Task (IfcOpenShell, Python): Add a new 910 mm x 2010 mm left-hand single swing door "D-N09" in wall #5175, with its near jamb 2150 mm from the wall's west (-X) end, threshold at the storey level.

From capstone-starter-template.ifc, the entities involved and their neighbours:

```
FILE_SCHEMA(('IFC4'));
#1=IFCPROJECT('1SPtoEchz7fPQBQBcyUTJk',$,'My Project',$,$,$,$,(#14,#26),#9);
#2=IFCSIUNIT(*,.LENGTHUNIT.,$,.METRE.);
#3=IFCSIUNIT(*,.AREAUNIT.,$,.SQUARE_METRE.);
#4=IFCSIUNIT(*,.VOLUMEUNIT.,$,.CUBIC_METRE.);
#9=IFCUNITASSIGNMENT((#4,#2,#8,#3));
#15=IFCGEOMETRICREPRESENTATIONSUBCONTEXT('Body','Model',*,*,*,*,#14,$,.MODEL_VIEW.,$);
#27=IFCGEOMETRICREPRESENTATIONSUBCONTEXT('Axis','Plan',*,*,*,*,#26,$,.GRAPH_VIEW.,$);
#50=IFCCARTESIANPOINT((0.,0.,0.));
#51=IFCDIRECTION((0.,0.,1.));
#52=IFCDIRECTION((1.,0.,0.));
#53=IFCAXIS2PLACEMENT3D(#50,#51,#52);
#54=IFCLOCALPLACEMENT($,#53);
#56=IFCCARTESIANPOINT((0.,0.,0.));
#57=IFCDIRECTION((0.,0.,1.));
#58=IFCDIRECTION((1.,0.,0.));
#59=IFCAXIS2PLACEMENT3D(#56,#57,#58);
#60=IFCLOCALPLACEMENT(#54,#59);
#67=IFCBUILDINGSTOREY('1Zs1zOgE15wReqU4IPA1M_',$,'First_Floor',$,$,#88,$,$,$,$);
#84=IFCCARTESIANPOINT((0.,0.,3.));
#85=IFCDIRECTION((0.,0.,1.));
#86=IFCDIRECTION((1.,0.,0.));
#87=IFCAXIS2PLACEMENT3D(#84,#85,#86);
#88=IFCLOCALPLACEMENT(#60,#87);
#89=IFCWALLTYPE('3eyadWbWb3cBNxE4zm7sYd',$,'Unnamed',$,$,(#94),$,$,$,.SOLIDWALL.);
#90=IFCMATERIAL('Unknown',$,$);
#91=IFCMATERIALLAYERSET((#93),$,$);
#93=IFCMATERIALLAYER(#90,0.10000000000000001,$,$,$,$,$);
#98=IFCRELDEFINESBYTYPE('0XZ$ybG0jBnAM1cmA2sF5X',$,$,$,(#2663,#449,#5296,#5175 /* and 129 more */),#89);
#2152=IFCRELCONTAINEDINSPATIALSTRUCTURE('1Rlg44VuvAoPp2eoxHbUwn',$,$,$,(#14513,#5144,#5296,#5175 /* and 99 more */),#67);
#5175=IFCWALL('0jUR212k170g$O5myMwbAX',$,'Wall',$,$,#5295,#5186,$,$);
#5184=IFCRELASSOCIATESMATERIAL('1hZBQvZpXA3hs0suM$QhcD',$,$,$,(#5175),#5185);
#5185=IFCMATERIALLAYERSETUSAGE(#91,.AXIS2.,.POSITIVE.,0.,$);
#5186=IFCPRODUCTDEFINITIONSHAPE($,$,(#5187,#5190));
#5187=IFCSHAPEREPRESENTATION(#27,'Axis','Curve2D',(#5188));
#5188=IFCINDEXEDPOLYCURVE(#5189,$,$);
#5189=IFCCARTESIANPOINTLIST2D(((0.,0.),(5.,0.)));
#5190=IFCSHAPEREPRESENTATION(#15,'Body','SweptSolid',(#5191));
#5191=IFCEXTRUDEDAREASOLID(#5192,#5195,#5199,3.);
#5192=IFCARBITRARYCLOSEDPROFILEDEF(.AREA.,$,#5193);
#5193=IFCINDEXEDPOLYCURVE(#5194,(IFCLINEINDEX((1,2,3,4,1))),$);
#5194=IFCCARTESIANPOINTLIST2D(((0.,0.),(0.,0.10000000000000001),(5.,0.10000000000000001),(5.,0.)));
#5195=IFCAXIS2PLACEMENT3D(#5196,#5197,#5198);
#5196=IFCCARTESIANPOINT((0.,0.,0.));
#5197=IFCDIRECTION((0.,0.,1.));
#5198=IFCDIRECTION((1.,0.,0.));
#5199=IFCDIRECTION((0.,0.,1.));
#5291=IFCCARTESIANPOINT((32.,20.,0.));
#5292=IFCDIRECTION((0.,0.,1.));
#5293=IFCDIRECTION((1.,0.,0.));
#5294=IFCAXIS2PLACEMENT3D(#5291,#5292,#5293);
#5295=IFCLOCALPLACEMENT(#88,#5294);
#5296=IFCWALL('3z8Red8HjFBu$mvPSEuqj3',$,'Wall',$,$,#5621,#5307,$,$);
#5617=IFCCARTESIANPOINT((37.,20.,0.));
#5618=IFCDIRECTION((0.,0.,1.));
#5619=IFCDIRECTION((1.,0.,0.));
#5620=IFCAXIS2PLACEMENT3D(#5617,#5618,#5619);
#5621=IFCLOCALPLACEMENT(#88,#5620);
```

```python
import numpy as np
import ifcopenshell
import ifcopenshell.api.feature
import ifcopenshell.api.geometry
import ifcopenshell.api.root
import ifcopenshell.api.spatial
import ifcopenshell.geom
import ifcopenshell.util.element
import ifcopenshell.util.placement
import ifcopenshell.util.representation
import ifcopenshell.util.shape
import ifcopenshell.util.unit

model = ifcopenshell.open("capstone-starter-template.ifc")
unit_scale = ifcopenshell.util.unit.calculate_unit_scale(model)
settings = ifcopenshell.geom.settings()


def volume(element):
    """Net volume in cubic metres, openings subtracted."""
    shape = ifcopenshell.geom.create_shape(settings, element)
    return ifcopenshell.util.shape.get_volume(shape.geometry)


wall = model.by_guid("0jUR212k170g$O5myMwbAX")
storey = ifcopenshell.util.element.get_container(wall, ifc_class="IfcBuildingStorey")
context = ifcopenshell.util.representation.get_context(model, "Model", "Body", "MODEL_VIEW")
before = volume(wall)

width, height, from_end, sill = 0.91, 2.01, 2.15, 0.0  # metres

# The wall runs along its own X axis, and the end named is its -X end.
wall_shape = ifcopenshell.geom.create_shape(settings, wall)
x, y, z = ifcopenshell.util.shape.get_vertices(wall_shape.geometry).T
start = x.min() + from_end
face, thickness = float(y.min()), float(y.max() - y.min())
wall_matrix = ifcopenshell.util.placement.get_local_placement(wall.ObjectPlacement)
level = ifcopenshell.util.placement.get_local_placement(storey.ObjectPlacement)[2, 3]


def in_wall(x, y):
    """Placement at x, y metres in the wall's axes, at sill height."""
    matrix = wall_matrix.copy()
    matrix[:, 3] = wall_matrix @ np.array([x / unit_scale, y / unit_scale, 0.0, 1.0])
    matrix[2, 3] = level + sill / unit_scale
    return matrix


# Opening: a box that overshoots both wall faces by 50 mm.
opening = ifcopenshell.api.root.create_entity(model, ifc_class="IfcOpeningElement", predefined_type="OPENING")
box = ifcopenshell.api.geometry.add_wall_representation(
    model, context=context, length=width, height=height, thickness=thickness + 0.1
)
ifcopenshell.api.geometry.assign_representation(model, product=opening, representation=box)
ifcopenshell.api.geometry.edit_object_placement(model, product=opening, matrix=in_wall(start, face - 0.05), is_si=False)
ifcopenshell.api.feature.add_feature(model, feature=opening, element=wall)

door = ifcopenshell.api.root.create_entity(model, ifc_class="IfcDoor", name="D-N09", predefined_type="DOOR")
door.OverallWidth, door.OverallHeight = width / unit_scale, height / unit_scale
door.OperationType = "SINGLE_SWING_LEFT"
body = ifcopenshell.api.geometry.add_door_representation(
    model,
    context=context,
    overall_width=door.OverallWidth,
    overall_height=door.OverallHeight,
    operation_type="SINGLE_SWING_LEFT",
    lining_properties={"LiningDepth": thickness / unit_scale, "ThresholdDepth": thickness / unit_scale},
)
ifcopenshell.api.geometry.assign_representation(model, product=door, representation=body)
ifcopenshell.api.spatial.assign_container(model, products=[door], relating_structure=storey)
ifcopenshell.api.feature.add_filling(model, opening=opening, element=door)

# The lining spans the wall, so the door starts at the wall face.
ifcopenshell.api.geometry.edit_object_placement(model, product=door, matrix=in_wall(start, face), is_si=False)

after = volume(wall)

print(f"wall volume {before:.3f} -> {after:.3f} m3")

model.write("capstone-starter-template-out.ifc")
```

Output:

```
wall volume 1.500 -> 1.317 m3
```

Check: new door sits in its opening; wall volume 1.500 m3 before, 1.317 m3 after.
